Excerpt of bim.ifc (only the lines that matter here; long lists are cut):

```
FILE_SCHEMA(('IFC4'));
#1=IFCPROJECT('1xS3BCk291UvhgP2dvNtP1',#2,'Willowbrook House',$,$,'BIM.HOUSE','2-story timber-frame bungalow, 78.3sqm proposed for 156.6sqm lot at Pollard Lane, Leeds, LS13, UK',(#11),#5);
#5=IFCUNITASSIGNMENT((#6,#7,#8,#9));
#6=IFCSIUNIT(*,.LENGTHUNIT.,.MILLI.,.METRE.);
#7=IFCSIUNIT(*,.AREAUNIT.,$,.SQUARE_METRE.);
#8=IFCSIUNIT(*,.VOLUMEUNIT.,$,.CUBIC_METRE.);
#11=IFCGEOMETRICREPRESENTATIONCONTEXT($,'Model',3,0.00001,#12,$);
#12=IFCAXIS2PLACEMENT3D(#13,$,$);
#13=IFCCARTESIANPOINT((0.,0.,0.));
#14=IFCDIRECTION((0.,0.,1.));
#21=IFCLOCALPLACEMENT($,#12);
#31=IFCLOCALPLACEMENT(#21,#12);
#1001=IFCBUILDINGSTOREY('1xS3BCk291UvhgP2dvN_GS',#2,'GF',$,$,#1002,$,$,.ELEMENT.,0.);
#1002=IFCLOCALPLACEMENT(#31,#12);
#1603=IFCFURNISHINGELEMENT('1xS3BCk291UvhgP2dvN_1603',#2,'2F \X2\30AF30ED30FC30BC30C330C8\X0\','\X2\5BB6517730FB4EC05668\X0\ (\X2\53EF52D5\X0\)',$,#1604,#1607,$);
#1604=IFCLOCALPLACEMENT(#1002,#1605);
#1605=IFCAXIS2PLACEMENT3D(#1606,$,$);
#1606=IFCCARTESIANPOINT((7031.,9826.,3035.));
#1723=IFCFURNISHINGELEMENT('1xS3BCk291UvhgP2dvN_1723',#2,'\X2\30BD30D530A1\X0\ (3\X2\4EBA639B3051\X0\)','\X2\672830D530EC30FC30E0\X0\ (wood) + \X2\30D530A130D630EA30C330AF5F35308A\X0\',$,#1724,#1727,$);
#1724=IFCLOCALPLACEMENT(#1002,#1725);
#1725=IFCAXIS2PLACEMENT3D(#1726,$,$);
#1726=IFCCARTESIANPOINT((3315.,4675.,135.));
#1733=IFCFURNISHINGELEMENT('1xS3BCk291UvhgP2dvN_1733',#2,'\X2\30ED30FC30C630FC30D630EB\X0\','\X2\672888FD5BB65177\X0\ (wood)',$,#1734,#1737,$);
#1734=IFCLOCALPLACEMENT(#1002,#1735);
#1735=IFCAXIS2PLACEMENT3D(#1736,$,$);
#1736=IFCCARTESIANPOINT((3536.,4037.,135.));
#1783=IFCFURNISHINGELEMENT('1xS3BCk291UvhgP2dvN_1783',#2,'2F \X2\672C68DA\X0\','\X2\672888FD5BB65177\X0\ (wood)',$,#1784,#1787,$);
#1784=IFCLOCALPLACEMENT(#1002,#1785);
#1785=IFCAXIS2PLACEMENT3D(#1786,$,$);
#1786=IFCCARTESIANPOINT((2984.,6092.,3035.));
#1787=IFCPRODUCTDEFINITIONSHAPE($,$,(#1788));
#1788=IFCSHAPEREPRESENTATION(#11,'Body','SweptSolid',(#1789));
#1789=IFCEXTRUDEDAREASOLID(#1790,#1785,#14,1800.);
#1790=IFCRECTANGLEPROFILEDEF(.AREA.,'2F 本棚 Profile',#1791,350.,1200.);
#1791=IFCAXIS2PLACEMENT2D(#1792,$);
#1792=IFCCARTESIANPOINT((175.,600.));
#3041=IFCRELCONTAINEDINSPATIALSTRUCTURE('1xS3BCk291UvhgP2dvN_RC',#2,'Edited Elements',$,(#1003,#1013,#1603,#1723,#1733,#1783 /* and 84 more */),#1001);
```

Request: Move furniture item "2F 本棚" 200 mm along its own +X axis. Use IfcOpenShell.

```python
import ifcopenshell
import ifcopenshell.api.geometry
import ifcopenshell.util.placement
import ifcopenshell.util.unit

model = ifcopenshell.open("bim.ifc")
unit_scale = ifcopenshell.util.unit.calculate_unit_scale(model)

item = model.by_guid("1xS3BCk291UvhgP2dvN_1783")
matrix = ifcopenshell.util.placement.get_local_placement(item.ObjectPlacement)
matrix[:3, 3] += matrix[:3, 0] * 0.2 / unit_scale
ifcopenshell.api.geometry.edit_object_placement(model, product=item, matrix=matrix, is_si=False)

print(ifcopenshell.util.placement.get_local_placement(item.ObjectPlacement).round(3) + 0.0)

model.write("bim_edited.ifc")
```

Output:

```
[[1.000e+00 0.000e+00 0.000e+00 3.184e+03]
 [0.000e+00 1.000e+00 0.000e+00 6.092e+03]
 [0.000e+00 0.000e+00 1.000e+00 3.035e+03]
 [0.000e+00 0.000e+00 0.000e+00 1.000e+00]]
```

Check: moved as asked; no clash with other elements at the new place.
